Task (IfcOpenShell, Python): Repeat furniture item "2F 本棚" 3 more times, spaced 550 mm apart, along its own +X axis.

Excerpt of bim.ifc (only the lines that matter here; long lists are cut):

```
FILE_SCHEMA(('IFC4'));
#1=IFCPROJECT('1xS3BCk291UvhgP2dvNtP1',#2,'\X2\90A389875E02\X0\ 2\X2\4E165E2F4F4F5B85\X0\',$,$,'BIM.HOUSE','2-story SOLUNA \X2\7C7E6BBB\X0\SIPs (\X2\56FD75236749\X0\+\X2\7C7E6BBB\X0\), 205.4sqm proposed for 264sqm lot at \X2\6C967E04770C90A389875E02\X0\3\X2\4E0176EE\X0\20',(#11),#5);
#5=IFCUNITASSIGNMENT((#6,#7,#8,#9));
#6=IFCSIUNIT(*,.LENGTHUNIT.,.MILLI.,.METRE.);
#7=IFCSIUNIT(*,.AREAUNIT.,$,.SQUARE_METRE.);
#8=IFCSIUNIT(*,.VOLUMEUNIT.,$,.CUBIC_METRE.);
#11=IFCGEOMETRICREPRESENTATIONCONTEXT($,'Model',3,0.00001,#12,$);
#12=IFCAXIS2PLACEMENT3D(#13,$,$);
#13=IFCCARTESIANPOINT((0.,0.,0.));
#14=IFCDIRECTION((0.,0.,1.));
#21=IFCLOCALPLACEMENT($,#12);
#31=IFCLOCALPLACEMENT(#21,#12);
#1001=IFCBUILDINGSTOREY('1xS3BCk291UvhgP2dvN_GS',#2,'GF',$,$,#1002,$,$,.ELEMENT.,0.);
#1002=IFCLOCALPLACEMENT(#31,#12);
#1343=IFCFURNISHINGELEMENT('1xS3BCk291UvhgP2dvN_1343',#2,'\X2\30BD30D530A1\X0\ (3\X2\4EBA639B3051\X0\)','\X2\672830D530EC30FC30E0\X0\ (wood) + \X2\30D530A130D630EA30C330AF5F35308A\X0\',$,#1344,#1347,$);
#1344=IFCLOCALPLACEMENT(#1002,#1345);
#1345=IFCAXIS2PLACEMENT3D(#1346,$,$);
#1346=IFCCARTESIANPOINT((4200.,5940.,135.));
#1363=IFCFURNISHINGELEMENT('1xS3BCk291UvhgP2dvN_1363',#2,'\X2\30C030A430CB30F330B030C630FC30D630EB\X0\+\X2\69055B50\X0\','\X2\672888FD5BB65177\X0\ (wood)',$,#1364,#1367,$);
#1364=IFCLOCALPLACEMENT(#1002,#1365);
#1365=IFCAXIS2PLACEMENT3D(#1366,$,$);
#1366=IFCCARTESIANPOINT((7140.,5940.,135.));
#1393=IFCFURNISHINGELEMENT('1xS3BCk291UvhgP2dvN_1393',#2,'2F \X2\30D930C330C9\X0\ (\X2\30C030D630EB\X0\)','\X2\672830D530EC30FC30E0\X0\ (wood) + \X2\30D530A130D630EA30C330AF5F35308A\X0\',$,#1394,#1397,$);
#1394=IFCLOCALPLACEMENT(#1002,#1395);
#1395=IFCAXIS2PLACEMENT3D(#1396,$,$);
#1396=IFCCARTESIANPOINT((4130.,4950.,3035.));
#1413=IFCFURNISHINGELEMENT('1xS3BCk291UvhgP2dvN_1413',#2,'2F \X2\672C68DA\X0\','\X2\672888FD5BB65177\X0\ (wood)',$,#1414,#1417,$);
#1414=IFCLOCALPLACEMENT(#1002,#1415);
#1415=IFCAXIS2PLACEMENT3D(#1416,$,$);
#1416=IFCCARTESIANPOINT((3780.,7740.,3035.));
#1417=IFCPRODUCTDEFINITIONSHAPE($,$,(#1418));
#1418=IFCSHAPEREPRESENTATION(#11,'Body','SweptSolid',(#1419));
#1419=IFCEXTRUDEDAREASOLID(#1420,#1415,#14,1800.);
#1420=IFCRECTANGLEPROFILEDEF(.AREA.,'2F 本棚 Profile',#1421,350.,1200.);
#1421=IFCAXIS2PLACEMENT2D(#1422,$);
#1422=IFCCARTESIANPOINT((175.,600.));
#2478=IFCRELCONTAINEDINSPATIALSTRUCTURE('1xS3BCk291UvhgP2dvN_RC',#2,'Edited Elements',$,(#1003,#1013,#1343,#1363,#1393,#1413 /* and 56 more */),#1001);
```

```python
import ifcopenshell
import ifcopenshell.api.geometry
import ifcopenshell.api.root
import ifcopenshell.util.element
import ifcopenshell.util.placement

model = ifcopenshell.open("bim.ifc")


def reuse_history(source, copy):
    """copy_class also copies each property set's owner history, people and application; keep the originals."""
    for rel in copy.IsDefinedBy:
        if rel.is_a("IfcRelDefinesByProperties") and (history := rel.RelatingPropertyDefinition.OwnerHistory):
            rel.RelatingPropertyDefinition.OwnerHistory = source.OwnerHistory
            ifcopenshell.util.element.remove_deep2(model, history)


source = model.by_guid("1xS3BCk291UvhgP2dvN_1413")
base = ifcopenshell.util.placement.get_local_placement(source.ObjectPlacement)
step = base[:3, 0] * 550.0

for i in range(1, 4):
    copy = ifcopenshell.api.root.copy_class(model, product=source)
    copy.Representation = ifcopenshell.util.element.copy_deep(
        model, source.Representation, exclude=["IfcGeometricRepresentationContext", "IfcRepresentationMap"]
    )
    reuse_history(source, copy)
    matrix = base.copy()
    matrix[:3, 3] += i * step
    print("added at", matrix[:3, 3].round(3) + 0.0)
    ifcopenshell.api.geometry.edit_object_placement(model, product=copy, matrix=matrix, is_si=False)

model.write("bim_rev.ifc")
```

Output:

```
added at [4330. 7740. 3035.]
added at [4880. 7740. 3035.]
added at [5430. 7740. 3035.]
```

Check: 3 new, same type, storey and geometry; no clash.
